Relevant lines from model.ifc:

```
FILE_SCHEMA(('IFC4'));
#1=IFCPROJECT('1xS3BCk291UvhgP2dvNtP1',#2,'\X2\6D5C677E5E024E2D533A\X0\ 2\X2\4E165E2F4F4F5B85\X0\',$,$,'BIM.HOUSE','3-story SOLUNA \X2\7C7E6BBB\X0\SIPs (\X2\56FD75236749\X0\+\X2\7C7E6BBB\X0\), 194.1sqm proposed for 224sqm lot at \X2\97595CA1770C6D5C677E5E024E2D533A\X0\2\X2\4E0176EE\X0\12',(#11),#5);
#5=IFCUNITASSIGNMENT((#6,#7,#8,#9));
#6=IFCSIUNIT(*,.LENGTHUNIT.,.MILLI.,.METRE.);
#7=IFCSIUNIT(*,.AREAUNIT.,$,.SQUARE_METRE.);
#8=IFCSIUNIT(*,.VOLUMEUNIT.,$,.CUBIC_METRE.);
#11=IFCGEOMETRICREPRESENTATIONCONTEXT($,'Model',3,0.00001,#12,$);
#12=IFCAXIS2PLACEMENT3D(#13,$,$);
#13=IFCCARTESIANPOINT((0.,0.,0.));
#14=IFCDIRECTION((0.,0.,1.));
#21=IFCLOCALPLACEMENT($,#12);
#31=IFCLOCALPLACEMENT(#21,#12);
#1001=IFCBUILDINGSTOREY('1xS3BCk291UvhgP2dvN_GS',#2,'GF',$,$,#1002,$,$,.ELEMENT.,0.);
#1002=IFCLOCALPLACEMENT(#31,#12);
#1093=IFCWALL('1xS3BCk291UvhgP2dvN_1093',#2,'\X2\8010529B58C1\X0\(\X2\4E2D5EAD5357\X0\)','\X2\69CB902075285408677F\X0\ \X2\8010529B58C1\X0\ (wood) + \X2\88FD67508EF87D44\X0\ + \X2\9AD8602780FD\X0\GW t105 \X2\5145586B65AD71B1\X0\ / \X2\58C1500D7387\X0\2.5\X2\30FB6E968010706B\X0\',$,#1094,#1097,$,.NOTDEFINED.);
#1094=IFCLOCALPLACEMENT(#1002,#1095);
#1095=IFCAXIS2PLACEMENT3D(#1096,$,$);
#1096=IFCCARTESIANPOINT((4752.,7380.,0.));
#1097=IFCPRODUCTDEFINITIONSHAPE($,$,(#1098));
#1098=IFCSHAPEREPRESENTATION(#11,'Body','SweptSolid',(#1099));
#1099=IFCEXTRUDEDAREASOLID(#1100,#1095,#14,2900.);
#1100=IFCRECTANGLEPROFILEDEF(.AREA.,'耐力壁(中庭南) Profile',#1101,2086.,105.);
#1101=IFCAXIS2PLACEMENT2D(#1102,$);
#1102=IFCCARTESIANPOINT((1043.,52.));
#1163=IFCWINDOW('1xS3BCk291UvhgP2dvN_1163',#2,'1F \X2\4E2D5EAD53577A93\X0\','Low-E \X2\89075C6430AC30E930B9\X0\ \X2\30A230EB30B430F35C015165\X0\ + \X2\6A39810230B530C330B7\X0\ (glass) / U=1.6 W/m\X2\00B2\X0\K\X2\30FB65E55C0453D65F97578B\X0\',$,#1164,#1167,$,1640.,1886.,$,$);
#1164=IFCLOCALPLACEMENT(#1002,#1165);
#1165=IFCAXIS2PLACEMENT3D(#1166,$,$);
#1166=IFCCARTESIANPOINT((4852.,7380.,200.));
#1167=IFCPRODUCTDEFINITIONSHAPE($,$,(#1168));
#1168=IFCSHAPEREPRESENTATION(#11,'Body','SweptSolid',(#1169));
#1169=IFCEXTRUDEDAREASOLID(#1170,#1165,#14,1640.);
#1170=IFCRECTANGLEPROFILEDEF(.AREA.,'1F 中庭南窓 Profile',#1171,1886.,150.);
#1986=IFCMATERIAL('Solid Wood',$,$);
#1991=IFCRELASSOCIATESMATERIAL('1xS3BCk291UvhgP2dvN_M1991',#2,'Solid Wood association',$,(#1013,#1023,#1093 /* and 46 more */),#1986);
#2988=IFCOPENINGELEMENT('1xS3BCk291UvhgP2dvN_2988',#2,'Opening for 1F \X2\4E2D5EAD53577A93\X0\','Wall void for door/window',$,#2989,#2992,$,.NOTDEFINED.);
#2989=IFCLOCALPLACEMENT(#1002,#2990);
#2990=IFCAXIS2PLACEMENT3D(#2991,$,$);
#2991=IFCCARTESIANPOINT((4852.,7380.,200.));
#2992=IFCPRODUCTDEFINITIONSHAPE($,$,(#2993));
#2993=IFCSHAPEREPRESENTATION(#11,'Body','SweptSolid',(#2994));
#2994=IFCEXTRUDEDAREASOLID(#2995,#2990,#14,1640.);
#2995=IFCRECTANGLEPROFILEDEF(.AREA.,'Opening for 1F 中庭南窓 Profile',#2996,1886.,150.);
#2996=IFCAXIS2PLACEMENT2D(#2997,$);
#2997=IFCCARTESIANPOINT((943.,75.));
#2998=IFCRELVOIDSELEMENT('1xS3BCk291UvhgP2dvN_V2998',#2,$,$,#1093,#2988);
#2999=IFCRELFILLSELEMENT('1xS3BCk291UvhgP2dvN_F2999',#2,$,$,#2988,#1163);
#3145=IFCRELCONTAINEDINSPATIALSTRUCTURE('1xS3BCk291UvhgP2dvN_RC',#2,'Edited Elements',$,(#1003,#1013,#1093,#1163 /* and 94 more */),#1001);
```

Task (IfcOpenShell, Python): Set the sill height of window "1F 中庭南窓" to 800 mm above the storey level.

```python
import numpy as np
import ifcopenshell
import ifcopenshell.api.geometry
import ifcopenshell.geom
import ifcopenshell.util.element
import ifcopenshell.util.placement
import ifcopenshell.util.shape
import ifcopenshell.util.unit

model = ifcopenshell.open("model.ifc")
unit_scale = ifcopenshell.util.unit.calculate_unit_scale(model)

window = model.by_guid("1xS3BCk291UvhgP2dvN_1163")
opening = window.FillsVoids[0].RelatingOpeningElement
storey = ifcopenshell.util.element.get_container(window, ifc_class="IfcBuildingStorey")
level = ifcopenshell.util.placement.get_local_placement(storey.ObjectPlacement)[2, 3]

# The opening's origin need not be at the sill, so measure its lowest point.
shape = ifcopenshell.geom.create_shape(ifcopenshell.geom.settings(), opening)
bottom = ifcopenshell.util.shape.get_shape_bottom_elevation(shape, shape.geometry) / unit_scale
dz = level + 0.8 / unit_scale - bottom

shift = np.array([0.0, 0.0, dz])
# The window is not placed relative to its opening, so move both.
for product in (opening, window):
    matrix = ifcopenshell.util.placement.get_local_placement(product.ObjectPlacement)
    matrix[:3, 3] += shift
    ifcopenshell.api.geometry.edit_object_placement(model, product=product, matrix=matrix, is_si=False)

print(f"moved by {dz * unit_scale:+.3f} m")

model.write("model_edited.ifc")
```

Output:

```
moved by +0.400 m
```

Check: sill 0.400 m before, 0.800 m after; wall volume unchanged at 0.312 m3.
